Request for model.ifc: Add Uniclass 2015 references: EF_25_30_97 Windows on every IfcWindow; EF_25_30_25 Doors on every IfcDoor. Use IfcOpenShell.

First a look at what the model holds.

```python
import ifcopenshell

model = ifcopenshell.open("model.ifc")
print(model.schema)
print("classifications:", [c.Name for c in model.by_type("IfcClassification")])
for ifc_class in ("IfcDoor", "IfcRoof", "IfcStair", "IfcWall", "IfcWindow"):
    print(ifc_class, len(model.by_type(ifc_class)))
```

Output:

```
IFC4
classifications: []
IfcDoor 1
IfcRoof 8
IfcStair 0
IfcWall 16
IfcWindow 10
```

```python
import ifcopenshell
import ifcopenshell.api.classification

model = ifcopenshell.open("model.ifc")

system = ifcopenshell.api.classification.add_classification(model, classification="Uniclass 2015")

codes = {
    "IfcWindow": ("EF_25_30_97", "Windows"),
    "IfcDoor": ("EF_25_30_25", "Doors"),
}
for ifc_class, (code, name) in codes.items():
    products = model.by_type(ifc_class)
    ifcopenshell.api.classification.add_reference(
        model, products=products, classification=system, identification=code, name=name
    )
    print(code, len(products))

model.write("model_updated.ifc")
```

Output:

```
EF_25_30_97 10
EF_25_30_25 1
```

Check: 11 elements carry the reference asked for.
